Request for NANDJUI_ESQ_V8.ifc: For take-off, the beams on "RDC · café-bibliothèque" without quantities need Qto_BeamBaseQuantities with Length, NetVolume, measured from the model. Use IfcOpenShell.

First a look at what the model holds.

```python
import ifcopenshell
import ifcopenshell.util.element
import ifcopenshell.util.unit

model = ifcopenshell.open("NANDJUI_ESQ_V8.ifc")
print(model.schema)
for unit_type in ("LENGTHUNIT", "AREAUNIT", "VOLUMEUNIT"):
    print(unit_type, ifcopenshell.util.unit.calculate_unit_scale(model, unit_type))
storey = next(s for s in model.by_type("IfcBuildingStorey") if s.Name == "RDC · café-bibliothèque")
beams = [e for e in ifcopenshell.util.element.get_decomposition(storey) if e.is_a("IfcBeam")]
for e in sorted(beams, key=lambda e: e.id()):
    print(e.id(), e.is_a(), e.Name, list(ifcopenshell.util.element.get_psets(e, qtos_only=True)), sep=" | ")
```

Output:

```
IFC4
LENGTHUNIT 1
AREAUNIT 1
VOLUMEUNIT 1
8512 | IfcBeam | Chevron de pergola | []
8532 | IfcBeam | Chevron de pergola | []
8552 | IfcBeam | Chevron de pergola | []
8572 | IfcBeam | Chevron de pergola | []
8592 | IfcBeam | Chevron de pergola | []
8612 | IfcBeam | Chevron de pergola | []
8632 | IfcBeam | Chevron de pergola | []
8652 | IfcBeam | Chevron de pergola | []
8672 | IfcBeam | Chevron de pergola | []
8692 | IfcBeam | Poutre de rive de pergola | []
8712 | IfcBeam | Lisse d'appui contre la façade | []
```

```python
import ifcopenshell
import ifcopenshell.api.pset
import ifcopenshell.geom
import ifcopenshell.util.element
import ifcopenshell.util.shape
import ifcopenshell.util.unit

model = ifcopenshell.open("NANDJUI_ESQ_V8.ifc")
unit_scale = ifcopenshell.util.unit.calculate_unit_scale(model)
volume_scale = ifcopenshell.util.unit.calculate_unit_scale(model, "VOLUMEUNIT")
settings = ifcopenshell.geom.settings()

storey = next(s for s in model.by_type("IfcBuildingStorey") if s.Name == "RDC · café-bibliothèque")
beams = [e for e in ifcopenshell.util.element.get_decomposition(storey) if e.is_a("IfcBeam")]

for e in sorted(beams, key=lambda e: e.id()):
    if ifcopenshell.util.element.get_psets(e, qtos_only=True, should_inherit=False):
        continue
    # Geometry comes back in metres, in the element's own axes.
    shape = ifcopenshell.geom.create_shape(settings, e)
    values = {
        "Length": ifcopenshell.util.shape.get_max_xyz(shape.geometry) / unit_scale,
        "NetVolume": ifcopenshell.util.shape.get_volume(shape.geometry) / volume_scale,
    }
    qto = ifcopenshell.api.pset.add_qto(model, product=e, name="Qto_BeamBaseQuantities")
    ifcopenshell.api.pset.edit_qto(model, qto=qto, properties=values)
    print(e.id(), {k: round(v, 3) for k, v in values.items()})

model.write("NANDJUI_ESQ_V8-out.ifc")
```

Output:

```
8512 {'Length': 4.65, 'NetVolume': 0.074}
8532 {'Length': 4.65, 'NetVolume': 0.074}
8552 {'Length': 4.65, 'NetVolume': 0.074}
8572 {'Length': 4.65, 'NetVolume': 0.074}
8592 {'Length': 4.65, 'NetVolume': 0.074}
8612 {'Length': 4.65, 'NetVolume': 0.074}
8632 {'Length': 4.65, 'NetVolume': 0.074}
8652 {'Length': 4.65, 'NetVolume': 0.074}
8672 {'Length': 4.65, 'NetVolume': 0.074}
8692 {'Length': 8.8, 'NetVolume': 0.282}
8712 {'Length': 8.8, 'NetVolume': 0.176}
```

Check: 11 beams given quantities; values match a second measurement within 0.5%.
